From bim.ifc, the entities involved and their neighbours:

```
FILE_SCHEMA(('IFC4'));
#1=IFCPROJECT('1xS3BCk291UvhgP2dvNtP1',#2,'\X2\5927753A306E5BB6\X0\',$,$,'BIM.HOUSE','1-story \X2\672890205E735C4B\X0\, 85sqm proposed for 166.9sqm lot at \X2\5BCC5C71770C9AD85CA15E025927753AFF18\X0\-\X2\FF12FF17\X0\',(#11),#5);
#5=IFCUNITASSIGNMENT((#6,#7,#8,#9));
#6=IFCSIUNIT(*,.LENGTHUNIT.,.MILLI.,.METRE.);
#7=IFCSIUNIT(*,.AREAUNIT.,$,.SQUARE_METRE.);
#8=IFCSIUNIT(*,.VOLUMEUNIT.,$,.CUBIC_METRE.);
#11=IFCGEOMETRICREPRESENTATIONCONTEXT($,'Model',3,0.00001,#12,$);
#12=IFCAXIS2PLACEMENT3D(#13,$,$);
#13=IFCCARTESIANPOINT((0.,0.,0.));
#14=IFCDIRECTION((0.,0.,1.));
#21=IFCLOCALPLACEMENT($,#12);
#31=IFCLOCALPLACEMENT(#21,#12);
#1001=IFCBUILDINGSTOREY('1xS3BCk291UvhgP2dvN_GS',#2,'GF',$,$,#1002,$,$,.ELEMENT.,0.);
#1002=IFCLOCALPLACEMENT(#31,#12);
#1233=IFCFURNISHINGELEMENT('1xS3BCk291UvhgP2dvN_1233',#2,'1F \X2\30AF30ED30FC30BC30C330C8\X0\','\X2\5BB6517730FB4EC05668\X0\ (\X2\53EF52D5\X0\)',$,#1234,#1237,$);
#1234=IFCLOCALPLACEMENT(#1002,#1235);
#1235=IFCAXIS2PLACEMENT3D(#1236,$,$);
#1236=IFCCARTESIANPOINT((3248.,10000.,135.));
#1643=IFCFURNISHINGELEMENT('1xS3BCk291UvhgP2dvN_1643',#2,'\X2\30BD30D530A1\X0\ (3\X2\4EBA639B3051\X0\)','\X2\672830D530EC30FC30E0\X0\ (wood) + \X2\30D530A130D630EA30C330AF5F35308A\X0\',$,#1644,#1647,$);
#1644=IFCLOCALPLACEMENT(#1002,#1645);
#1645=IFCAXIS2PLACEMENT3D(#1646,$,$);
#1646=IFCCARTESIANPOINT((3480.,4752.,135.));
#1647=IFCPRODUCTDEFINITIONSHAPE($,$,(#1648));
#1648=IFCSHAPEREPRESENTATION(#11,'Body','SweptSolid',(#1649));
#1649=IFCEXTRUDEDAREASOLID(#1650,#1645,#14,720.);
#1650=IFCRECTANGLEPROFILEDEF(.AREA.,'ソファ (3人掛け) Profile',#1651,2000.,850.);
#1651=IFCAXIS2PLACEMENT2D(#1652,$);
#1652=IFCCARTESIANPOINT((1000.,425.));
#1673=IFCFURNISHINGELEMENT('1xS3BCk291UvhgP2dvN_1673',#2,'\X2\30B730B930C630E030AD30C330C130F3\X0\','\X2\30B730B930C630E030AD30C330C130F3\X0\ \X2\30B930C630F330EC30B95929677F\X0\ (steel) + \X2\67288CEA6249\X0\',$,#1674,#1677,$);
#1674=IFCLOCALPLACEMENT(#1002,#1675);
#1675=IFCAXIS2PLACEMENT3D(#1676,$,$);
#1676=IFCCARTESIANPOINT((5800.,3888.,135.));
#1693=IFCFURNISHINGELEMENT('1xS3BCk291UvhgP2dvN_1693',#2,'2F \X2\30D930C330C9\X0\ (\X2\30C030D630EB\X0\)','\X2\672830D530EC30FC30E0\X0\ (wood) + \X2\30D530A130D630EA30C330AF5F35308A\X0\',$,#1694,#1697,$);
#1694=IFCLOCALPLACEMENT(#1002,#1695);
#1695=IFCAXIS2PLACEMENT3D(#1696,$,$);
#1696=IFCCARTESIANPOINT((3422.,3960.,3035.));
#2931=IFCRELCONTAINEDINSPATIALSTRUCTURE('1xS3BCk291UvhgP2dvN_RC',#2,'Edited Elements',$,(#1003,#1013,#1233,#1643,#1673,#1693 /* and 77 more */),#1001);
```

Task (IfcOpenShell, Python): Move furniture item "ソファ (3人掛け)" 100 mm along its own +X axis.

```python
import ifcopenshell
import ifcopenshell.api.geometry
import ifcopenshell.util.placement
import ifcopenshell.util.unit

model = ifcopenshell.open("bim.ifc")
unit_scale = ifcopenshell.util.unit.calculate_unit_scale(model)

item = model.by_guid("1xS3BCk291UvhgP2dvN_1643")
matrix = ifcopenshell.util.placement.get_local_placement(item.ObjectPlacement)
matrix[:3, 3] += matrix[:3, 0] * 0.1 / unit_scale
ifcopenshell.api.geometry.edit_object_placement(model, product=item, matrix=matrix, is_si=False)

print(ifcopenshell.util.placement.get_local_placement(item.ObjectPlacement).round(3) + 0.0)

model.write("bim_edited.ifc")
```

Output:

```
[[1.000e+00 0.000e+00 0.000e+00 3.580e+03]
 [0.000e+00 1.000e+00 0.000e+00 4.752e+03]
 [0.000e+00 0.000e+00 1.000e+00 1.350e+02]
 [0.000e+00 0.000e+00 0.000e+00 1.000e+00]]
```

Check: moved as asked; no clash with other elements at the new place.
